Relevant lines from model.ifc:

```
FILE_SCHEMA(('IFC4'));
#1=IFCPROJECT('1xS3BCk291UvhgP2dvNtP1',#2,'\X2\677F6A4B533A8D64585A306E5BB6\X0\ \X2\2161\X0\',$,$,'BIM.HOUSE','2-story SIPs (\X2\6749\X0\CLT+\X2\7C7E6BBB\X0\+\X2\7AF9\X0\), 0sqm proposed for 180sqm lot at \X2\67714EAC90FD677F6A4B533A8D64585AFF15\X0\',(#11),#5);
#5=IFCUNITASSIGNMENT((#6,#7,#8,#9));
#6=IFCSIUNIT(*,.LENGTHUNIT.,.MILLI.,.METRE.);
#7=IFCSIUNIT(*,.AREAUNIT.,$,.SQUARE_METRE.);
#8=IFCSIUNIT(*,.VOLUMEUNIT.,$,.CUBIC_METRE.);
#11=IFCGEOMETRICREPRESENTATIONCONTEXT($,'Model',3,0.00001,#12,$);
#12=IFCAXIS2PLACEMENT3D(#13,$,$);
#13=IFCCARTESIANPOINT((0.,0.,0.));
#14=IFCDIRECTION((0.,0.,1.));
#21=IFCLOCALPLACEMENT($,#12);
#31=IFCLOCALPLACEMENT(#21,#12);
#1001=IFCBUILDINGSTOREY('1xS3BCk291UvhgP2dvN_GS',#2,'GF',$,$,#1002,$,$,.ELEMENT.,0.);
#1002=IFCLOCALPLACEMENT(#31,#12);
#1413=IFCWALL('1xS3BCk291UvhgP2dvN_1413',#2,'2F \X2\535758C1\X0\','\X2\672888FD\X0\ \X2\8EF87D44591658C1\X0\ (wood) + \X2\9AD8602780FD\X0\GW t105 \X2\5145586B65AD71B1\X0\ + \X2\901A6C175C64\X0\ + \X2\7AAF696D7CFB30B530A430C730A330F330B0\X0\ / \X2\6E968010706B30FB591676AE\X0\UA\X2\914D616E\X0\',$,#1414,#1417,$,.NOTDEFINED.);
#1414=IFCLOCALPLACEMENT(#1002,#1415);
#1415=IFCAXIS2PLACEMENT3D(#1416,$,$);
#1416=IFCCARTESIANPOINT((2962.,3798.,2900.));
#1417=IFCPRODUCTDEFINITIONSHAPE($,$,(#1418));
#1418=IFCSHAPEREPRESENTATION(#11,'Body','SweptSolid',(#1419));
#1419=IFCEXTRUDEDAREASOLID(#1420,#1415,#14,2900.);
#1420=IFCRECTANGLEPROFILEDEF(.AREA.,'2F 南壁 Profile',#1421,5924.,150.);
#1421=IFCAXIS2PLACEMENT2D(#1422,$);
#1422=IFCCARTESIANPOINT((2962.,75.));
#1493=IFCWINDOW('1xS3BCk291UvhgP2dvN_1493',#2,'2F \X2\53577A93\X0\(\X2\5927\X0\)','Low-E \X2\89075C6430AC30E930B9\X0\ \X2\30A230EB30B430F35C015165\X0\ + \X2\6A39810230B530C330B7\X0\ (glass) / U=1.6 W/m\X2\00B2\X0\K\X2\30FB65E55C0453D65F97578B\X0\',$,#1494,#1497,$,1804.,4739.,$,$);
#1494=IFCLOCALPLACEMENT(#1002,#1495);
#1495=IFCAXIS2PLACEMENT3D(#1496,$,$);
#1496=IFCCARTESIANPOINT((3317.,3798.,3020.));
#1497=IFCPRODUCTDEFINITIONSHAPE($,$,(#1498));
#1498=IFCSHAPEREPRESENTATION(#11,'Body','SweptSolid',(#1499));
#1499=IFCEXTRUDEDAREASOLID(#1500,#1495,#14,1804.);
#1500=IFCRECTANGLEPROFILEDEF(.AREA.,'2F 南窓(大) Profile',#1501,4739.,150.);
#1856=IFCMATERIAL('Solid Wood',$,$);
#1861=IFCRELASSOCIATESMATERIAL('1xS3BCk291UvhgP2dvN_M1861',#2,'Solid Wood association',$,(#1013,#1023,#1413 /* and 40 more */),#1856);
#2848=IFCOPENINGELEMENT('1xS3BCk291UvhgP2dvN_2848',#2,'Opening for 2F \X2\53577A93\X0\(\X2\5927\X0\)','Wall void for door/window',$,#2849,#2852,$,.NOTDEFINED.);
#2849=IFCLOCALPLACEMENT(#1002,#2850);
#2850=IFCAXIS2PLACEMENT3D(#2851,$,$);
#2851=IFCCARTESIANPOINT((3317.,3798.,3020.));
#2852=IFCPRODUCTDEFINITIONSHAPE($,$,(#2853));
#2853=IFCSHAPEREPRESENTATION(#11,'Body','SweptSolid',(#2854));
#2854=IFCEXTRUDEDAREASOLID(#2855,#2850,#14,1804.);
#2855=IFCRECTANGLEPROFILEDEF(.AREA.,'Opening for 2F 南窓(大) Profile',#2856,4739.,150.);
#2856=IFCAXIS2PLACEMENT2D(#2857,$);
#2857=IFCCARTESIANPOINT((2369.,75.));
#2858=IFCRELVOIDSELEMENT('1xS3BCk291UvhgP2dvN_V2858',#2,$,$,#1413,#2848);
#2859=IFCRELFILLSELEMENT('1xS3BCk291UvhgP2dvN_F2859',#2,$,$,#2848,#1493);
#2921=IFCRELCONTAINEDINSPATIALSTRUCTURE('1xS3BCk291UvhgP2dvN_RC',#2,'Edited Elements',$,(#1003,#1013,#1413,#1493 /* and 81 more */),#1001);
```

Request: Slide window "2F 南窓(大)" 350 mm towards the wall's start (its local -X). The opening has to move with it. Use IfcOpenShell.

```python
import ifcopenshell
import ifcopenshell.api.geometry
import ifcopenshell.util.placement
import ifcopenshell.util.unit

model = ifcopenshell.open("model.ifc")
unit_scale = ifcopenshell.util.unit.calculate_unit_scale(model)

window = model.by_id(1493)
opening = window.FillsVoids[0].RelatingOpeningElement
wall = opening.VoidsElements[0].RelatingBuildingElement

wall_matrix = ifcopenshell.util.placement.get_local_placement(wall.ObjectPlacement)
shift = wall_matrix[:3, 0] * -0.35 / unit_scale
before = ifcopenshell.util.placement.get_local_placement(window.ObjectPlacement)[:3, 3].copy()

# The window is not placed relative to its opening, so move both.
for product in (opening, window):
    matrix = ifcopenshell.util.placement.get_local_placement(product.ObjectPlacement)
    matrix[:3, 3] += shift
    ifcopenshell.api.geometry.edit_object_placement(model, product=product, matrix=matrix, is_si=False)

after = ifcopenshell.util.placement.get_local_placement(window.ObjectPlacement)[:3, 3]
print("window moved by", (after - before).round(3) + 0.0)

model.write("model-out.ifc")
```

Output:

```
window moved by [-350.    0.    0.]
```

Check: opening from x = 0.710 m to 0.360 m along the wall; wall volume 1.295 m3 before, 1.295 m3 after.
